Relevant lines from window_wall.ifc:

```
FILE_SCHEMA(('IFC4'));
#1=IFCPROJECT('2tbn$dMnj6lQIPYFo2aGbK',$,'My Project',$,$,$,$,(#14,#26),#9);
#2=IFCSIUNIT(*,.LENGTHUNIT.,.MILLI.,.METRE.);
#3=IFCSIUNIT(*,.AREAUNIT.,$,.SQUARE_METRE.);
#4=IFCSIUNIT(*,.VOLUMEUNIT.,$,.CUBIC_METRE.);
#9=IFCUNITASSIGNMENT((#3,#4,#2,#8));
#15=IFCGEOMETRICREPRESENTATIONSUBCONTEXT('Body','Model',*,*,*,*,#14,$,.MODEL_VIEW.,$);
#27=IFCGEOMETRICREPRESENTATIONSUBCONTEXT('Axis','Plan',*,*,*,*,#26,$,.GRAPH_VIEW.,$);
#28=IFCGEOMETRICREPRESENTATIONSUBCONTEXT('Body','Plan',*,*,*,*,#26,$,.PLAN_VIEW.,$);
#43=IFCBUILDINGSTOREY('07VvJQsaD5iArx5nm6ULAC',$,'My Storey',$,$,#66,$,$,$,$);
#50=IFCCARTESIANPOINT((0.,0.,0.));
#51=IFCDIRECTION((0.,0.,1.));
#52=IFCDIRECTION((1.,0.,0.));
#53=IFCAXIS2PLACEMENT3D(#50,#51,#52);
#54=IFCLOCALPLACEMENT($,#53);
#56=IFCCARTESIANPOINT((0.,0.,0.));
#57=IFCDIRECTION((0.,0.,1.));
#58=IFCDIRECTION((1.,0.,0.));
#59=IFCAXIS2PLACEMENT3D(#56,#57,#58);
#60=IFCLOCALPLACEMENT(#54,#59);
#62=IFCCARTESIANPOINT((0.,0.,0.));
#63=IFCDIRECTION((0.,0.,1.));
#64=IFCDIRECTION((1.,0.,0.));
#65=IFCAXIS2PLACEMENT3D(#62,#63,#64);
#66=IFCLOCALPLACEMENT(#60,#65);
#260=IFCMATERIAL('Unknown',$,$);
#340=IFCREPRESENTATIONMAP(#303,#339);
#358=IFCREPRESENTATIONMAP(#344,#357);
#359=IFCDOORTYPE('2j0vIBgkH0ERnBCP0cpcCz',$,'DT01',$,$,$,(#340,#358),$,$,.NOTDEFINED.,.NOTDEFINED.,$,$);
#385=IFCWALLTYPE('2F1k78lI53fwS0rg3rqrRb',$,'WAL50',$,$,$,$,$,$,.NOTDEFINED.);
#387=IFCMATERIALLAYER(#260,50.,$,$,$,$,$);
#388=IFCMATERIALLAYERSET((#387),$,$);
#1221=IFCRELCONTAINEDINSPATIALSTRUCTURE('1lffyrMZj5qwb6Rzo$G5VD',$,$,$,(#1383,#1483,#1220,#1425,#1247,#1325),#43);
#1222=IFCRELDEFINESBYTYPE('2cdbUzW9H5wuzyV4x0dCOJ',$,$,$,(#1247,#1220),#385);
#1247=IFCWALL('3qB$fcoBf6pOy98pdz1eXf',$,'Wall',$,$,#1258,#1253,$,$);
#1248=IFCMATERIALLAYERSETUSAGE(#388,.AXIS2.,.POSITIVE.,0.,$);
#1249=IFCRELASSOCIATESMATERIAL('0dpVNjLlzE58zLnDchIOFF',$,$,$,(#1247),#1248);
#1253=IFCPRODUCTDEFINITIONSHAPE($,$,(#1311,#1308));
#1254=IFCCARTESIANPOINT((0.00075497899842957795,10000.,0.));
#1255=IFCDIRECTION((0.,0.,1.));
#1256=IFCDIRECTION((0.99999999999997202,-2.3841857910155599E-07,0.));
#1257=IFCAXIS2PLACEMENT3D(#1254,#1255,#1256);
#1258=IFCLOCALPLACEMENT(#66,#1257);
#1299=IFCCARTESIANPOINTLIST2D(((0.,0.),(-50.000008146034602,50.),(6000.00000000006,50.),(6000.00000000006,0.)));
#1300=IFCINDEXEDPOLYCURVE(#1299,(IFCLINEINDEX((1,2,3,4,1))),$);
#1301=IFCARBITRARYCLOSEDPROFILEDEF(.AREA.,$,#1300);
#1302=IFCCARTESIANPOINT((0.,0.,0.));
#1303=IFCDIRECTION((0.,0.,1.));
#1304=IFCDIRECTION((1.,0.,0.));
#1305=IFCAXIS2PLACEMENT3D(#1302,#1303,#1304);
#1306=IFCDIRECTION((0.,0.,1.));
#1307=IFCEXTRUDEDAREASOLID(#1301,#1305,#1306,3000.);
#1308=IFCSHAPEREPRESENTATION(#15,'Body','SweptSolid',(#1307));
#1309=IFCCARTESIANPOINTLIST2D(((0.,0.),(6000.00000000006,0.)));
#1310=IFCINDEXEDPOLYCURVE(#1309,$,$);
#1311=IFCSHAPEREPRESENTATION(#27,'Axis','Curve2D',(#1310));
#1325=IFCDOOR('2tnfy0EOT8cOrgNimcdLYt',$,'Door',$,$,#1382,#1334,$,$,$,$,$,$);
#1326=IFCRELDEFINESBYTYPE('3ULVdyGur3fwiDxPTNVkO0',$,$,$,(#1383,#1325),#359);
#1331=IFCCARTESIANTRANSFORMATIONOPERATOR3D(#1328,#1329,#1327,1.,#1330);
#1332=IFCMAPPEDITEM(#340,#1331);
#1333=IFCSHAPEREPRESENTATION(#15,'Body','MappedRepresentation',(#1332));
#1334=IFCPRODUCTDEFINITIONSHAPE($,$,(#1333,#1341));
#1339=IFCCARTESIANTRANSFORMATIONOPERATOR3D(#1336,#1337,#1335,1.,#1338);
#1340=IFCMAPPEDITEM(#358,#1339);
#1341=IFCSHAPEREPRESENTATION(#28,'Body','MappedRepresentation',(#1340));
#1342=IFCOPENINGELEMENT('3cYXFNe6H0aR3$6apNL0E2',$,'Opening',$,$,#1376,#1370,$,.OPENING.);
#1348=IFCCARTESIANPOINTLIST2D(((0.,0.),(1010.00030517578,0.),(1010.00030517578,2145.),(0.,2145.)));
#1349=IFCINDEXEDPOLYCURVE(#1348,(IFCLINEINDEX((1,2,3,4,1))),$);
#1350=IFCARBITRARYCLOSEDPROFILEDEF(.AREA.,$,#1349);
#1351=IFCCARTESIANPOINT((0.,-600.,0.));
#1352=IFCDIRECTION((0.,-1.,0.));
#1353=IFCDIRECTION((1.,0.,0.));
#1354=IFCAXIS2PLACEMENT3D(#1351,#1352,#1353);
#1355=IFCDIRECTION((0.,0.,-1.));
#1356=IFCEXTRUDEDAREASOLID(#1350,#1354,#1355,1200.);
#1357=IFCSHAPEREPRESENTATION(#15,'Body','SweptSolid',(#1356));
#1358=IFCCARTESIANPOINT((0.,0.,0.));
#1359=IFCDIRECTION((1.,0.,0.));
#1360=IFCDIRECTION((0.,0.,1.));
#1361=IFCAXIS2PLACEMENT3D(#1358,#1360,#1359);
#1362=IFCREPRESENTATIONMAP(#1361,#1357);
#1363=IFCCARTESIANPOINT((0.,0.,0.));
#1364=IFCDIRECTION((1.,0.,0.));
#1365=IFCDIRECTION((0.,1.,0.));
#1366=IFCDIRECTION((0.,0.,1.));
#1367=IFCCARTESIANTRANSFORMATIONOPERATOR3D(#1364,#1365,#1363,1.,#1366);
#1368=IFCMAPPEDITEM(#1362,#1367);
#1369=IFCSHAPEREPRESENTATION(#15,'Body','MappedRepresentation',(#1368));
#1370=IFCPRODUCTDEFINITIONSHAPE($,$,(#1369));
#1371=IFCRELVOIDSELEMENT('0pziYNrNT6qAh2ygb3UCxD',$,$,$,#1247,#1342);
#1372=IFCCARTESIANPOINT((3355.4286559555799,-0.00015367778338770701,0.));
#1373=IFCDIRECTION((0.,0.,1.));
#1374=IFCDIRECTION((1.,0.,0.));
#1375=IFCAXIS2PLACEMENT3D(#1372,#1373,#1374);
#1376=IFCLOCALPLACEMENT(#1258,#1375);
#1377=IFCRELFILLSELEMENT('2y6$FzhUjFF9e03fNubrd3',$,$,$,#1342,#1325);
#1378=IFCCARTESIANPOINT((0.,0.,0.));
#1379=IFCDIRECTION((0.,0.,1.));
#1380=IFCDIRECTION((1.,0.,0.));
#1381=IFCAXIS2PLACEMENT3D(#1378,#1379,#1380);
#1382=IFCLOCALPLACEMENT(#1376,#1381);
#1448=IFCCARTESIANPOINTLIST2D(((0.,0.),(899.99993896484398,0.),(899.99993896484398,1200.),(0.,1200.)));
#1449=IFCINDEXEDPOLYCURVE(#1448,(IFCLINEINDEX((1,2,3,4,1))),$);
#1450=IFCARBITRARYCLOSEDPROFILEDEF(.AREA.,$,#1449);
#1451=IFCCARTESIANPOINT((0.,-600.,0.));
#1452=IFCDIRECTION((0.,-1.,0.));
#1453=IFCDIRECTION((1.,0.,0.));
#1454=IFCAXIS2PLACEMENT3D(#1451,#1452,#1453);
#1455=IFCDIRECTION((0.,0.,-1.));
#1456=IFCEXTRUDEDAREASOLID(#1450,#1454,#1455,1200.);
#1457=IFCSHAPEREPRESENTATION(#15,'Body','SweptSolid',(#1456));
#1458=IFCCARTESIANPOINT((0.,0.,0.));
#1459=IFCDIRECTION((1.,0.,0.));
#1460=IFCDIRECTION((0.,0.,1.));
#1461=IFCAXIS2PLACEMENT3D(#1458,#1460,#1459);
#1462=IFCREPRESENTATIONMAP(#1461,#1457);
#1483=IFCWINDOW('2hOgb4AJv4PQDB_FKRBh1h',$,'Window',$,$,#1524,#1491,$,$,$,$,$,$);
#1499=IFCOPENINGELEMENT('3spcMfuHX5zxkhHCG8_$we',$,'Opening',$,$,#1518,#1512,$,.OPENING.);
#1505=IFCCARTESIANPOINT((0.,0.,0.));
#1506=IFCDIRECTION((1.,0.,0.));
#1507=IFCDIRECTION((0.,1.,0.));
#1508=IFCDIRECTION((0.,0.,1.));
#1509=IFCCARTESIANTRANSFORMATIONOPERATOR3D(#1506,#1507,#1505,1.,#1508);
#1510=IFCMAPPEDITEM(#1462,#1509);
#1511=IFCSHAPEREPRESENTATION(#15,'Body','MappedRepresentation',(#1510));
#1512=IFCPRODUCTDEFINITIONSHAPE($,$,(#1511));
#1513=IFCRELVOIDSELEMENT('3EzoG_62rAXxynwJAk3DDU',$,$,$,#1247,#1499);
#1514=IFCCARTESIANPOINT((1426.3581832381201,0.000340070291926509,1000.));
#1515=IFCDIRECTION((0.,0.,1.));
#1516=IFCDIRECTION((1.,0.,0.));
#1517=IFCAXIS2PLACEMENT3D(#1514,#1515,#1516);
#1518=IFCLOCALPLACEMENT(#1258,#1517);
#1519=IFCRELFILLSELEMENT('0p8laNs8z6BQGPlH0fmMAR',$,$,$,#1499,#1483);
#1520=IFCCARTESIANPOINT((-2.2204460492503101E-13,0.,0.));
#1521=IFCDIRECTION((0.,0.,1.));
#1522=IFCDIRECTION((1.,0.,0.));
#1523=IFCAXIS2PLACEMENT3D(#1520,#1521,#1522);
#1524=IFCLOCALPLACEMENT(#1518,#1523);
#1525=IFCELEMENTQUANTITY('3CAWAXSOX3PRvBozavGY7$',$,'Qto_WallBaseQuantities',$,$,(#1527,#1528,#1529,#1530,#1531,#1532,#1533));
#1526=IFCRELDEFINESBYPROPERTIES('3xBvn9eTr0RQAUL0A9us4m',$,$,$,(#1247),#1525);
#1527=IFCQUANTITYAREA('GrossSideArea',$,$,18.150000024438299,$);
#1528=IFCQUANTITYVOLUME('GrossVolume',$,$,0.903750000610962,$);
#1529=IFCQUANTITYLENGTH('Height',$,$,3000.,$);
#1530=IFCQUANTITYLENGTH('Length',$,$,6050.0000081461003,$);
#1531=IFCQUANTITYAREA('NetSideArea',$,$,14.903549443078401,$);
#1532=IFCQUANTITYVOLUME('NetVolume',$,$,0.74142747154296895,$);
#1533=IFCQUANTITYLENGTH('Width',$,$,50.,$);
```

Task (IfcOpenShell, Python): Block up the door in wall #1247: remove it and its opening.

```python
import ifcopenshell
import ifcopenshell.api.feature
import ifcopenshell.api.pset
import ifcopenshell.api.root
import ifcopenshell.geom
import ifcopenshell.util.element
import ifcopenshell.util.shape
import ifcopenshell.util.unit

model = ifcopenshell.open("window_wall.ifc")
area_scale = ifcopenshell.util.unit.calculate_unit_scale(model, "AREAUNIT")
volume_scale = ifcopenshell.util.unit.calculate_unit_scale(model, "VOLUMEUNIT")
settings = ifcopenshell.geom.settings()


def volume(element):
    """Net volume in cubic metres, openings subtracted."""
    shape = ifcopenshell.geom.create_shape(settings, element)
    return ifcopenshell.util.shape.get_volume(shape.geometry)


door = model.by_id(1325)
opening = door.FillsVoids[0].RelatingOpeningElement
wall = opening.VoidsElements[0].RelatingBuildingElement
before = volume(wall)

ifcopenshell.api.root.remove_product(model, product=door)
ifcopenshell.api.feature.remove_feature(model, feature=opening)

after = volume(wall)
thickness = 0.05  # wall thickness in metres

# Update the wall's stored quantities.
qto = model.by_id(ifcopenshell.util.element.get_pset(wall, "Qto_WallBaseQuantities", should_inherit=False)["id"])
ifcopenshell.api.pset.edit_qto(model, qto=qto, properties={
    "NetSideArea": after / thickness / area_scale,
    "NetVolume": after / volume_scale,
})

print(f"wall volume {before:.3f} -> {after:.3f} m3")

model.write("window_wall-out.ifc")
```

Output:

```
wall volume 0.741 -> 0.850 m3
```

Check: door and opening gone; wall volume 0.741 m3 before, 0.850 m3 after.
